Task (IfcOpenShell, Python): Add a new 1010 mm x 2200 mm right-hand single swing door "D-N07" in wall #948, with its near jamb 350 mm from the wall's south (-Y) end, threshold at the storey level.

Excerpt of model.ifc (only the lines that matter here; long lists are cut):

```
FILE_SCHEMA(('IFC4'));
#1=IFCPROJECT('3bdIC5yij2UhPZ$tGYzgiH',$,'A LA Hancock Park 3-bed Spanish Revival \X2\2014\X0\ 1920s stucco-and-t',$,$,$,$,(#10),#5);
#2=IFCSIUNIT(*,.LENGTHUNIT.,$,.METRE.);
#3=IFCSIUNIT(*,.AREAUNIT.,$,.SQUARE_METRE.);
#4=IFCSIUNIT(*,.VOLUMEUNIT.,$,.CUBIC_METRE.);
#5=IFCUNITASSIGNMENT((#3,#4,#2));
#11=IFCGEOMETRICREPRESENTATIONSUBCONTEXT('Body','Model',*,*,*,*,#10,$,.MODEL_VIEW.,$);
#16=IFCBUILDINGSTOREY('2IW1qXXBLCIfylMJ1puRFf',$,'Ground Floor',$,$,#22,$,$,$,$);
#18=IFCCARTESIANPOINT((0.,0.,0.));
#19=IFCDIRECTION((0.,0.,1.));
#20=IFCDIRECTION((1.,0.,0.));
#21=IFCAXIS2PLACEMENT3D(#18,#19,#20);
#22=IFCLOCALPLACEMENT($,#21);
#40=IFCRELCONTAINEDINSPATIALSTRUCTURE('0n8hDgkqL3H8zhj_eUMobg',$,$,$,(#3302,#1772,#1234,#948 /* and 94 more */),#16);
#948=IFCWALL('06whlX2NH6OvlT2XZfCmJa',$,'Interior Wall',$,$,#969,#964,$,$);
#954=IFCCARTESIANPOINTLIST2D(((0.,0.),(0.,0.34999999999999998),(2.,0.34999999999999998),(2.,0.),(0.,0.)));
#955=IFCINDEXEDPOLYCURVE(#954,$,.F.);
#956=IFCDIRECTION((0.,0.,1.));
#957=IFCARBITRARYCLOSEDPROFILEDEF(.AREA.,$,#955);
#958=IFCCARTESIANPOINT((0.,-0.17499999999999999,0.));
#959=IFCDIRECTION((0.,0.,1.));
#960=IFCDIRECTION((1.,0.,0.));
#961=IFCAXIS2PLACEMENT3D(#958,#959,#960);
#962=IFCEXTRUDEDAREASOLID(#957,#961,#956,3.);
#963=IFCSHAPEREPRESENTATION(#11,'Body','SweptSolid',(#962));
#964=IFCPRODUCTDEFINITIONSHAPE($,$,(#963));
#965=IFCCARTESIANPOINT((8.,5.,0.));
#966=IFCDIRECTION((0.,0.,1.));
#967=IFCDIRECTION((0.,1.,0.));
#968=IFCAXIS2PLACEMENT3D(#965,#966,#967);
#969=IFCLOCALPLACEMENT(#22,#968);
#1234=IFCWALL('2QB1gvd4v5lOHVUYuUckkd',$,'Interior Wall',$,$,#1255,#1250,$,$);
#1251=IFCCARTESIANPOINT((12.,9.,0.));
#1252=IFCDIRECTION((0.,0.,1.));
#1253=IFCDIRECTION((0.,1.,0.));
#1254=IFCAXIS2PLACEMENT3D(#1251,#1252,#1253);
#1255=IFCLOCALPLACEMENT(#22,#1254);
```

```python
import numpy as np
import ifcopenshell
import ifcopenshell.api.feature
import ifcopenshell.api.geometry
import ifcopenshell.api.root
import ifcopenshell.api.spatial
import ifcopenshell.geom
import ifcopenshell.util.element
import ifcopenshell.util.placement
import ifcopenshell.util.representation
import ifcopenshell.util.shape
import ifcopenshell.util.unit

model = ifcopenshell.open("model.ifc")
unit_scale = ifcopenshell.util.unit.calculate_unit_scale(model)
settings = ifcopenshell.geom.settings()


def volume(element):
    """Net volume in cubic metres, openings subtracted."""
    shape = ifcopenshell.geom.create_shape(settings, element)
    return ifcopenshell.util.shape.get_volume(shape.geometry)


wall = model.by_guid("06whlX2NH6OvlT2XZfCmJa")
storey = ifcopenshell.util.element.get_container(wall, ifc_class="IfcBuildingStorey")
context = ifcopenshell.util.representation.get_context(model, "Model", "Body", "MODEL_VIEW")
before = volume(wall)

width, height, from_end, sill = 1.01, 2.2, 0.35, 0.0  # metres

# The wall runs along its own X axis, and the end named is its -X end.
wall_shape = ifcopenshell.geom.create_shape(settings, wall)
x, y, z = ifcopenshell.util.shape.get_vertices(wall_shape.geometry).T
start = x.min() + from_end
face, thickness = float(y.min()), float(y.max() - y.min())
wall_matrix = ifcopenshell.util.placement.get_local_placement(wall.ObjectPlacement)
level = ifcopenshell.util.placement.get_local_placement(storey.ObjectPlacement)[2, 3]


def in_wall(x, y):
    """Placement at x, y metres in the wall's axes, at sill height."""
    matrix = wall_matrix.copy()
    matrix[:, 3] = wall_matrix @ np.array([x / unit_scale, y / unit_scale, 0.0, 1.0])
    matrix[2, 3] = level + sill / unit_scale
    return matrix


# Opening: a box that overshoots both wall faces by 50 mm.
opening = ifcopenshell.api.root.create_entity(model, ifc_class="IfcOpeningElement", predefined_type="OPENING")
box = ifcopenshell.api.geometry.add_wall_representation(
    model, context=context, length=width, height=height, thickness=thickness + 0.1
)
ifcopenshell.api.geometry.assign_representation(model, product=opening, representation=box)
ifcopenshell.api.geometry.edit_object_placement(model, product=opening, matrix=in_wall(start, face - 0.05), is_si=False)
ifcopenshell.api.feature.add_feature(model, feature=opening, element=wall)

door = ifcopenshell.api.root.create_entity(model, ifc_class="IfcDoor", name="D-N07", predefined_type="DOOR")
door.OverallWidth, door.OverallHeight = width / unit_scale, height / unit_scale
door.OperationType = "SINGLE_SWING_RIGHT"
body = ifcopenshell.api.geometry.add_door_representation(
    model,
    context=context,
    overall_width=door.OverallWidth,
    overall_height=door.OverallHeight,
    operation_type="SINGLE_SWING_RIGHT",
    lining_properties={"LiningDepth": thickness / unit_scale, "ThresholdDepth": thickness / unit_scale},
)
ifcopenshell.api.geometry.assign_representation(model, product=door, representation=body)
ifcopenshell.api.spatial.assign_container(model, products=[door], relating_structure=storey)
ifcopenshell.api.feature.add_filling(model, opening=opening, element=door)

# The lining spans the wall, so the door starts at the wall face.
ifcopenshell.api.geometry.edit_object_placement(model, product=door, matrix=in_wall(start, face), is_si=False)

after = volume(wall)

print(f"wall volume {before:.3f} -> {after:.3f} m3")

model.write("model_v2.ifc")
```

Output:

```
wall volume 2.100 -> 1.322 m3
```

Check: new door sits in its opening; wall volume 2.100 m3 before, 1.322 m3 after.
